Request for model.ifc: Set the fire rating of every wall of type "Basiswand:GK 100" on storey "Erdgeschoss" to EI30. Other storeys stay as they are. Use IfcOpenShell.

First a look at what the model holds.

```python
import ifcopenshell
import ifcopenshell.util.element

model = ifcopenshell.open("model.ifc")
print(model.schema)
storey = next(s for s in model.by_type("IfcBuildingStorey") if s.Name == "Erdgeschoss")
walls = [e for e in ifcopenshell.util.element.get_decomposition(storey) if e.is_a("IfcWall")]
seen = {}
for e in walls:
    element_type = ifcopenshell.util.element.get_type(e)
    key = (element_type.Name if element_type != e and element_type else None, ifcopenshell.util.element.get_pset(e, "Pset_WallCommon", "FireRating"))
    seen[key] = seen.get(key, 0) + 1
for (name, value), count in sorted(seen.items(), key=str):
    print(count, "x", name, "|", value)
```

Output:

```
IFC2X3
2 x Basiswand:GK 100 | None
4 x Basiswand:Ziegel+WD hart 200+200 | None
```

```python
import ifcopenshell
import ifcopenshell.api.pset
import ifcopenshell.util.element

model = ifcopenshell.open("model.ifc")

storey = next(s for s in model.by_type("IfcBuildingStorey") if s.Name == "Erdgeschoss")
walls = [e for e in ifcopenshell.util.element.get_decomposition(storey) if e.is_a("IfcWall")]

count = 0
for e in walls:
    element_type = ifcopenshell.util.element.get_type(e)
    if element_type in (None, e) or element_type.Name != "Basiswand:GK 100":
        continue
    # add_pset returns the element's existing set when there is one.
    pset = ifcopenshell.api.pset.add_pset(model, product=e, name="Pset_WallCommon")
    ifcopenshell.api.pset.edit_pset(model, pset=pset, properties={"FireRating": "EI30"})
    count += 1

print(count, "walls updated")

model.write("model_rev.ifc")
```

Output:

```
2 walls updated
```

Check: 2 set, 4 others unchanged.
